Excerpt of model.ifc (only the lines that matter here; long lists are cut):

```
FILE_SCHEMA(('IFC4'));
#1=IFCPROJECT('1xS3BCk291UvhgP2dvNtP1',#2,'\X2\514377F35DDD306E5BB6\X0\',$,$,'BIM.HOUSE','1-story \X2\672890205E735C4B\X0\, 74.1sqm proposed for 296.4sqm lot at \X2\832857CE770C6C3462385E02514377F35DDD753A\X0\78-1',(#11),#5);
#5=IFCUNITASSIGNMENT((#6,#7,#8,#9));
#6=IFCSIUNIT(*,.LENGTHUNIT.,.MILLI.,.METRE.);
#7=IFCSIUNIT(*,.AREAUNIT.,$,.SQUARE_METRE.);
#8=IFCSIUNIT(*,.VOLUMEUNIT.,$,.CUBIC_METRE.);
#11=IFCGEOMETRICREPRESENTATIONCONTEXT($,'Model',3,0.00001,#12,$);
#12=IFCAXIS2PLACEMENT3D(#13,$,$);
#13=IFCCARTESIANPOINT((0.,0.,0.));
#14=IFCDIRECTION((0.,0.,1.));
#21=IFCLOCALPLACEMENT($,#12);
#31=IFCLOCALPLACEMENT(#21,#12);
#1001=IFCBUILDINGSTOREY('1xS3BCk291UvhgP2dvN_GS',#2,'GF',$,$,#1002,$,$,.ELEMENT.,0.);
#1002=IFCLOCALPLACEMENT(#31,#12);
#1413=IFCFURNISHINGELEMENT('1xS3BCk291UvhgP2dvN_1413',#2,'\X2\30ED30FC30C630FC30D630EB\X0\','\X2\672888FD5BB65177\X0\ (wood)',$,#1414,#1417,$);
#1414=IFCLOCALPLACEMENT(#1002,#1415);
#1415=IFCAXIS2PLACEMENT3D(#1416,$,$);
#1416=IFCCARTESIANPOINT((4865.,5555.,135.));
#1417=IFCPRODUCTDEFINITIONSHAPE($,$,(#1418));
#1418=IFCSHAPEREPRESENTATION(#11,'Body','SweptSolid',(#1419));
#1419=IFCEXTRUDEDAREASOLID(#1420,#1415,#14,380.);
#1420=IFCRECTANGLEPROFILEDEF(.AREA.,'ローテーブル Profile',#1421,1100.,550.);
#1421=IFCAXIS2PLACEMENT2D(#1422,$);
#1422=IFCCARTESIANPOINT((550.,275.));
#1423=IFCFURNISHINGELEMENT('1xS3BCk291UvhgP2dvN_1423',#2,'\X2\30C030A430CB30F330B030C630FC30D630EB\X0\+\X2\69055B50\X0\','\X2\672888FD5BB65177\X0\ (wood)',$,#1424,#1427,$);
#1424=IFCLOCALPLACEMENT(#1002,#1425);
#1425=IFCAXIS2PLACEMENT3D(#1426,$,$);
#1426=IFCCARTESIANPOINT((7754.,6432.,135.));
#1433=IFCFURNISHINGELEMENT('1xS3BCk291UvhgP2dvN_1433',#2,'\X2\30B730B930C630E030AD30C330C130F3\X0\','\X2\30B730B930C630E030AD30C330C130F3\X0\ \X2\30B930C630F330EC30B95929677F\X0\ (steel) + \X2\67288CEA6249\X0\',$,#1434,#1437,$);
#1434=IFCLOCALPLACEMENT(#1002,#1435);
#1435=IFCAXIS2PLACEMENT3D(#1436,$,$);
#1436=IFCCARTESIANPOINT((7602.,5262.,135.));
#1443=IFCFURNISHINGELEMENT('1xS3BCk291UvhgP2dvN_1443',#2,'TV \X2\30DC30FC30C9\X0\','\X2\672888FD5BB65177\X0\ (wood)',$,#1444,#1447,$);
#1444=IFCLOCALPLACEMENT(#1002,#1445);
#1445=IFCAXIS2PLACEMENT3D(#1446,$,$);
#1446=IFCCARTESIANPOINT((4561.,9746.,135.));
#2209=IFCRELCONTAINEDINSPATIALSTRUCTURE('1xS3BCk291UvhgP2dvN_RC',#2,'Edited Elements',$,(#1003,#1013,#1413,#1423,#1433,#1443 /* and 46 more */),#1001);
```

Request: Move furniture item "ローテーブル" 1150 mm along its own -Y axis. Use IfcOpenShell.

```python
import ifcopenshell
import ifcopenshell.api.geometry
import ifcopenshell.util.placement
import ifcopenshell.util.unit

model = ifcopenshell.open("model.ifc")
unit_scale = ifcopenshell.util.unit.calculate_unit_scale(model)

item = model.by_id(1413)
matrix = ifcopenshell.util.placement.get_local_placement(item.ObjectPlacement)
matrix[:3, 3] -= matrix[:3, 1] * 1.15 / unit_scale
ifcopenshell.api.geometry.edit_object_placement(model, product=item, matrix=matrix, is_si=False)

print(ifcopenshell.util.placement.get_local_placement(item.ObjectPlacement).round(3) + 0.0)

model.write("model_updated.ifc")
```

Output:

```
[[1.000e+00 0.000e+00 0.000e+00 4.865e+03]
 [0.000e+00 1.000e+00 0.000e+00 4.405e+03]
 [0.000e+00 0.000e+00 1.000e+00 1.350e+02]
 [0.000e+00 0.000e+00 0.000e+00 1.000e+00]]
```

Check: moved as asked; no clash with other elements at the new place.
